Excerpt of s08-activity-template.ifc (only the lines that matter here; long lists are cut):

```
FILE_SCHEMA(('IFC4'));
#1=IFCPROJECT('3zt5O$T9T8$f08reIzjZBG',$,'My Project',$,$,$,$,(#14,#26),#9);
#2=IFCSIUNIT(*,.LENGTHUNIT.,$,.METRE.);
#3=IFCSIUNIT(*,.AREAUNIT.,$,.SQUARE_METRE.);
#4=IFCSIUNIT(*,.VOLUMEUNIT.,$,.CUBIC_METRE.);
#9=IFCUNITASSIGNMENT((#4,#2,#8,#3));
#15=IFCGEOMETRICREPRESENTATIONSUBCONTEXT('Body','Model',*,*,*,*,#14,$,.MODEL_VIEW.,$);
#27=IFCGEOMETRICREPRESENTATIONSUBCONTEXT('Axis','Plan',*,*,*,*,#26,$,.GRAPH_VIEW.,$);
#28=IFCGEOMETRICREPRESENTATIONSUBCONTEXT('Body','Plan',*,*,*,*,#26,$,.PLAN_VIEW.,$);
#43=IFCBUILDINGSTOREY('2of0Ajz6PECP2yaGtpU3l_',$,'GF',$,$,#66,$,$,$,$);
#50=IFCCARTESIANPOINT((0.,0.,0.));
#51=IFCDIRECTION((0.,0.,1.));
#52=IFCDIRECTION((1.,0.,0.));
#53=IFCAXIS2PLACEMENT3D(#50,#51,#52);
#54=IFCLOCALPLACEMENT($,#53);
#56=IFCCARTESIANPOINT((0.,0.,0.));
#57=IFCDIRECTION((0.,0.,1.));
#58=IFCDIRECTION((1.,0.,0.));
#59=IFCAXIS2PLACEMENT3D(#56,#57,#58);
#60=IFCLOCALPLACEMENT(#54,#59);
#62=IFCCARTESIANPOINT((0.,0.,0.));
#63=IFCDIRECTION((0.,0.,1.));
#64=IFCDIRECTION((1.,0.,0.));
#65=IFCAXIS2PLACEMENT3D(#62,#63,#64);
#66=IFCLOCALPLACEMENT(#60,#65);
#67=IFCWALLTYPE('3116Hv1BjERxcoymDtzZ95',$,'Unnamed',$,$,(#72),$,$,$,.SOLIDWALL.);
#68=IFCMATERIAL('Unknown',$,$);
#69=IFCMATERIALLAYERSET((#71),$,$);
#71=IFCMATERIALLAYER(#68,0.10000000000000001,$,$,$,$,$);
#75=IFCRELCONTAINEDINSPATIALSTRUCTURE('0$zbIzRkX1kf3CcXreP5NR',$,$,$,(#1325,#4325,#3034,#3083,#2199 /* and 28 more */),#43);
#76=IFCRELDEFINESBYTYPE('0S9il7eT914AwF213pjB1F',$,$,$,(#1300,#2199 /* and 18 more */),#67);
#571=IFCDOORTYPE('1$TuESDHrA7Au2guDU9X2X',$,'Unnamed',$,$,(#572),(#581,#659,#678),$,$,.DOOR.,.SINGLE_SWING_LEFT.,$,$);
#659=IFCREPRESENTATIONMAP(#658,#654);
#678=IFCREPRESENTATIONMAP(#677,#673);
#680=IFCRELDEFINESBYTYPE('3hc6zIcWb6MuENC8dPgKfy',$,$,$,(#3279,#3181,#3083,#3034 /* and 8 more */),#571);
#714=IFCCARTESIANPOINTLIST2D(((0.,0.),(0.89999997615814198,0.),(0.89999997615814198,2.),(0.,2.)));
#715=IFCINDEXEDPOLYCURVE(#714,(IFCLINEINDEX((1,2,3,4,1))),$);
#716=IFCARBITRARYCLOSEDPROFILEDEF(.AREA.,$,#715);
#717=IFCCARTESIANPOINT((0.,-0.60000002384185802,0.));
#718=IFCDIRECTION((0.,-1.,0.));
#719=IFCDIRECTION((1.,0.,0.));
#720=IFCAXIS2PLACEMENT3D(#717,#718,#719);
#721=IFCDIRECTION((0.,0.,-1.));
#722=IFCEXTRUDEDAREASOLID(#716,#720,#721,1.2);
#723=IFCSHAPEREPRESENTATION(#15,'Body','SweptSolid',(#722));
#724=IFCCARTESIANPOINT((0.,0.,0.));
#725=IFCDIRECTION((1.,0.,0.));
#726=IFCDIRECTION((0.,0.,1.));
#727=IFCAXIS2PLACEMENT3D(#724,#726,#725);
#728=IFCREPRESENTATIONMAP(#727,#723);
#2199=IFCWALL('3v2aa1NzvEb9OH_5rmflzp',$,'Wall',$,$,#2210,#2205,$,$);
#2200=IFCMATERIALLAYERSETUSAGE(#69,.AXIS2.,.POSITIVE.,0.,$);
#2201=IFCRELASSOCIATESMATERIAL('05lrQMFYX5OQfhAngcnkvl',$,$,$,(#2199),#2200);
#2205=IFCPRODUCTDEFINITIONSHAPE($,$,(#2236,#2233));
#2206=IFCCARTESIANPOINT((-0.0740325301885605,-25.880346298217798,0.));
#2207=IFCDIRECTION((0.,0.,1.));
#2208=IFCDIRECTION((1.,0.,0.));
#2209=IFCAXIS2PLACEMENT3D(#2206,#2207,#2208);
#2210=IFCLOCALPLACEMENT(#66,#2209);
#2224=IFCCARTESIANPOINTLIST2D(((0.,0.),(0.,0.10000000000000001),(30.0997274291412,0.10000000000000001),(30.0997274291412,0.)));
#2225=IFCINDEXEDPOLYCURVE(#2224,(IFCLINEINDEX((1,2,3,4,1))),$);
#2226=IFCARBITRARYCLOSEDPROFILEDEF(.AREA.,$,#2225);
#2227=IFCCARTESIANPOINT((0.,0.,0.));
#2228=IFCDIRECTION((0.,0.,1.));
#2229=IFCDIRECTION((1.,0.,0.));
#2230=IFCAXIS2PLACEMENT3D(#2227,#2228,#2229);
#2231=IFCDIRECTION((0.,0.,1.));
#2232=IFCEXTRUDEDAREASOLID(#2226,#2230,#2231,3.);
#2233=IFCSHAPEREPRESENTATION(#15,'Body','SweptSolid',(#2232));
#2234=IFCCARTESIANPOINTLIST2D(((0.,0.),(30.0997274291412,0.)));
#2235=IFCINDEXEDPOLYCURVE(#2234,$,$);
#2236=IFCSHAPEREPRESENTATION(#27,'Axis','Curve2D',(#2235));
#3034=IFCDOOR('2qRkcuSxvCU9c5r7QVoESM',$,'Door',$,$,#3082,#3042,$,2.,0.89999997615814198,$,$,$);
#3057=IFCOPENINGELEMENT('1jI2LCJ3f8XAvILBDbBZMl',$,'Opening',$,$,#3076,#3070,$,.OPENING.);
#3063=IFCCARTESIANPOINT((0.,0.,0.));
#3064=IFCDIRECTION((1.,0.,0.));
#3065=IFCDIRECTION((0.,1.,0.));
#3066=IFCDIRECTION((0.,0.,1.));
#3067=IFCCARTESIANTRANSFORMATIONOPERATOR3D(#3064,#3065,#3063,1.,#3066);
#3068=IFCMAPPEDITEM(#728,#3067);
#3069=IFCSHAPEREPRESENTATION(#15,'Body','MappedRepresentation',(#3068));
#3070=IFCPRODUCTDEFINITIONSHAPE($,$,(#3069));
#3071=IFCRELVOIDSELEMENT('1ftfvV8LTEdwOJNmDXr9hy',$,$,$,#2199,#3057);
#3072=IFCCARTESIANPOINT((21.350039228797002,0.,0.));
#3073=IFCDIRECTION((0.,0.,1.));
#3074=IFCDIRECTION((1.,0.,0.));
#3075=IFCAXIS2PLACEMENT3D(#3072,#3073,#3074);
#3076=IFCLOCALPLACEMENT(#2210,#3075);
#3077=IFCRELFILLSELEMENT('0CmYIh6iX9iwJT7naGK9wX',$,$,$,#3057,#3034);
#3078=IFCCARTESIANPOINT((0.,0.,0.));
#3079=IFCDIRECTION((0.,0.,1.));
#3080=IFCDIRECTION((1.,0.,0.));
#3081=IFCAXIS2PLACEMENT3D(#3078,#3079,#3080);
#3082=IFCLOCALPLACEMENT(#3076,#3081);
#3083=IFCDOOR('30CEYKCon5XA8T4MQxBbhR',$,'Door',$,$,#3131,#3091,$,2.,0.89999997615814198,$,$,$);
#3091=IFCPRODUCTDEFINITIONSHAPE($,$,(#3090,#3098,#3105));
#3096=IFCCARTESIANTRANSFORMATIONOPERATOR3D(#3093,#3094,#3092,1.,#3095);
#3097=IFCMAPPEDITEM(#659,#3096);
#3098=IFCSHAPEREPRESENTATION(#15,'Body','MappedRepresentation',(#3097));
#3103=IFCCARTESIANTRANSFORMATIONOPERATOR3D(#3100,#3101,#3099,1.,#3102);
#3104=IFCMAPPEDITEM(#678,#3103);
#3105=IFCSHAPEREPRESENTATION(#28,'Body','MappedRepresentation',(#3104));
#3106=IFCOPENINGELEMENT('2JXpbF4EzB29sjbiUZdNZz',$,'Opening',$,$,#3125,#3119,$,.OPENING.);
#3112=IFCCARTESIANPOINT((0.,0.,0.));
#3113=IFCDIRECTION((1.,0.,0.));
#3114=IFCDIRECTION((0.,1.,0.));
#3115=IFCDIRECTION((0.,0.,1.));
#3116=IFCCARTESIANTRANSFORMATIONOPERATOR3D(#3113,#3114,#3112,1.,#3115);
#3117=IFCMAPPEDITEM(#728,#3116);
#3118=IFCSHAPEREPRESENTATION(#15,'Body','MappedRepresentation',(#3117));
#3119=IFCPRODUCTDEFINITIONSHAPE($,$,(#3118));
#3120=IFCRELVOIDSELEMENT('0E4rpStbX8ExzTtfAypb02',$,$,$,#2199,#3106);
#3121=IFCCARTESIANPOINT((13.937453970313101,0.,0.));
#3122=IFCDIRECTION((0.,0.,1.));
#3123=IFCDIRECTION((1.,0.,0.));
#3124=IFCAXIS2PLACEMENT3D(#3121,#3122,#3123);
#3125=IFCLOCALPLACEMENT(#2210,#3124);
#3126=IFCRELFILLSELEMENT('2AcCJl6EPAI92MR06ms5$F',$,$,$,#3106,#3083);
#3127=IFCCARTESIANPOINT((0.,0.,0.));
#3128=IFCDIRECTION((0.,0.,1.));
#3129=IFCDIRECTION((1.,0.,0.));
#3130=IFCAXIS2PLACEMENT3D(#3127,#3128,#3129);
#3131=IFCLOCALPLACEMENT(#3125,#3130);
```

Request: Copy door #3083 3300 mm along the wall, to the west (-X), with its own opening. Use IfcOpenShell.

```python
import ifcopenshell
import ifcopenshell.api.feature
import ifcopenshell.api.geometry
import ifcopenshell.api.root
import ifcopenshell.geom
import ifcopenshell.util.element
import ifcopenshell.util.placement
import ifcopenshell.util.shape
import ifcopenshell.util.unit

model = ifcopenshell.open("s08-activity-template.ifc")
unit_scale = ifcopenshell.util.unit.calculate_unit_scale(model)
settings = ifcopenshell.geom.settings()


def volume(element):
    """Net volume in cubic metres, openings subtracted."""
    shape = ifcopenshell.geom.create_shape(settings, element)
    return ifcopenshell.util.shape.get_volume(shape.geometry)


door = model.by_guid("30CEYKCon5XA8T4MQxBbhR")
opening = door.FillsVoids[0].RelatingOpeningElement
wall = opening.VoidsElements[0].RelatingBuildingElement
before = volume(wall)
shift = ifcopenshell.util.placement.get_local_placement(wall.ObjectPlacement)[:3, 0] * -3.3 / unit_scale

# copy_class copies the void relationship, type, container and properties, but no geometry.
new_opening = ifcopenshell.api.root.copy_class(model, product=opening)
new_opening.Representation = ifcopenshell.util.element.copy_deep(
    model, opening.Representation, exclude=["IfcGeometricRepresentationContext", "IfcRepresentationMap"]
)
new_door = ifcopenshell.api.root.copy_class(model, product=door)
new_door.Representation = ifcopenshell.util.element.copy_deep(
    model, door.Representation, exclude=["IfcGeometricRepresentationContext", "IfcRepresentationMap"]
)
ifcopenshell.api.feature.add_filling(model, opening=new_opening, element=new_door)

for old, new in ((opening, new_opening), (door, new_door)):
    matrix = ifcopenshell.util.placement.get_local_placement(old.ObjectPlacement)
    matrix[:3, 3] += shift
    ifcopenshell.api.geometry.edit_object_placement(model, product=new, matrix=matrix, is_si=False)

after = volume(wall)

print(f"wall volume {before:.3f} -> {after:.3f} m3")

model.write("s08-activity-template_rev.ifc")
```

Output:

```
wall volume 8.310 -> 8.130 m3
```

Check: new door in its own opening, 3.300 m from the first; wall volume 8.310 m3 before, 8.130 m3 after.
